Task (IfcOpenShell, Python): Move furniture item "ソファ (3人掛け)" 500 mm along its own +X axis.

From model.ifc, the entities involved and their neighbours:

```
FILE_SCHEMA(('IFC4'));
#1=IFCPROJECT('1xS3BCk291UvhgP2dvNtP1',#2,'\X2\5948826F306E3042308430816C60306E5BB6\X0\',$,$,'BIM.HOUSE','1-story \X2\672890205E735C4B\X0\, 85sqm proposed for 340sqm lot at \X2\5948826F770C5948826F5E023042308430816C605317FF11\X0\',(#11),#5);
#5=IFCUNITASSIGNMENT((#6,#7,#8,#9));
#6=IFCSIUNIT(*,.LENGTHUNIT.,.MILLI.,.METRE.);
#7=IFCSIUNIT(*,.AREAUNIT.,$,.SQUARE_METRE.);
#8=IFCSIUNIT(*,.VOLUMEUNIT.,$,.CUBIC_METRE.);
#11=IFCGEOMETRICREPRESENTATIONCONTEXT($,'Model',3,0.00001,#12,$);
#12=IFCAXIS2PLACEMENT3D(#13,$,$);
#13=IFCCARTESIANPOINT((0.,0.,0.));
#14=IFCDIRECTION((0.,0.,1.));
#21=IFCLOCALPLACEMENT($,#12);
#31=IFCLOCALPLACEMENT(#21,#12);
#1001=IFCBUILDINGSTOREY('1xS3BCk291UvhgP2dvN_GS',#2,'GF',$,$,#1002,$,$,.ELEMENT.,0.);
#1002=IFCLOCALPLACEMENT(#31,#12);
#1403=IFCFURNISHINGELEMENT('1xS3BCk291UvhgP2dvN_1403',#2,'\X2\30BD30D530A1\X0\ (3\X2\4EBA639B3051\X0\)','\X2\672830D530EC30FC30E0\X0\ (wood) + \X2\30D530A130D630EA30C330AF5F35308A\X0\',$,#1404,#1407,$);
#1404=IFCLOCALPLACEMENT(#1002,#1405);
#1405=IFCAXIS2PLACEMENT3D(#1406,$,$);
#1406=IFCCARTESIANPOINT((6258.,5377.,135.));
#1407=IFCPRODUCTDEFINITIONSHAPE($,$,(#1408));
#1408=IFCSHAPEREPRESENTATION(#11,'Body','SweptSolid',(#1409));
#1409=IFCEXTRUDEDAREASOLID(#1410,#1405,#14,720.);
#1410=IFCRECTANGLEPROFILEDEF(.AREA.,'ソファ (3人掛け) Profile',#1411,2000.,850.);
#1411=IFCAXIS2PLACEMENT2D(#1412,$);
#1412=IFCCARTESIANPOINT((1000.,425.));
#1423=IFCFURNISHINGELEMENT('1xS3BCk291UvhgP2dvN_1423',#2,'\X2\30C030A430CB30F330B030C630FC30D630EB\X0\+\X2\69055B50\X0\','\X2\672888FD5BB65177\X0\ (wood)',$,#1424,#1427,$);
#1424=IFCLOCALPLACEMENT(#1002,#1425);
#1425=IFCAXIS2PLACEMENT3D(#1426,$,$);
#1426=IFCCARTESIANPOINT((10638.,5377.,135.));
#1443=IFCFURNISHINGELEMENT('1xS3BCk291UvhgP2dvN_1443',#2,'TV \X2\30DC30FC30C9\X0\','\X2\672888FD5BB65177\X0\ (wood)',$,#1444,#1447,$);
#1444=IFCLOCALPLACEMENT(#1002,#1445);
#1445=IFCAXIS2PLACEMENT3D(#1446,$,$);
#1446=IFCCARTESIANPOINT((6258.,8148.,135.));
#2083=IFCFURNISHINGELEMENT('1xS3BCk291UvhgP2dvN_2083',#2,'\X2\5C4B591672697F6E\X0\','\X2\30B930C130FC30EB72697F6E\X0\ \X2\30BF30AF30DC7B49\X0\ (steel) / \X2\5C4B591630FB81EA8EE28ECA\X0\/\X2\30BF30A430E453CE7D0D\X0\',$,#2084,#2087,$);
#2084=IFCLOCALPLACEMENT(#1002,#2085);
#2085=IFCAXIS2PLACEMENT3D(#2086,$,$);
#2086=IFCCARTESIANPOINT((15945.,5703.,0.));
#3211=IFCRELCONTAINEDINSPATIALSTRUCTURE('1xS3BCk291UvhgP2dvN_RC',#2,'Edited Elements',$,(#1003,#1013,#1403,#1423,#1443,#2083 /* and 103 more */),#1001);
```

```python
import ifcopenshell
import ifcopenshell.api.geometry
import ifcopenshell.util.placement
import ifcopenshell.util.unit

model = ifcopenshell.open("model.ifc")
unit_scale = ifcopenshell.util.unit.calculate_unit_scale(model)

item = model.by_guid("1xS3BCk291UvhgP2dvN_1403")
matrix = ifcopenshell.util.placement.get_local_placement(item.ObjectPlacement)
matrix[:3, 3] += matrix[:3, 0] * 0.5 / unit_scale
ifcopenshell.api.geometry.edit_object_placement(model, product=item, matrix=matrix, is_si=False)

print(ifcopenshell.util.placement.get_local_placement(item.ObjectPlacement).round(3) + 0.0)

model.write("model-out.ifc")
```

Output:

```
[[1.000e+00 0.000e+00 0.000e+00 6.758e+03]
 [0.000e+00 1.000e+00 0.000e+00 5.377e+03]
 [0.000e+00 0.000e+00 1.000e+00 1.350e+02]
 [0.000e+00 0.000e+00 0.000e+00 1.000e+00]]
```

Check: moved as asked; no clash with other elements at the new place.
